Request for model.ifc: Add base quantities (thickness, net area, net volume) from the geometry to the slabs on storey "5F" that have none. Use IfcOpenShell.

First a look at what the model holds.

```python
import ifcopenshell
import ifcopenshell.util.element
import ifcopenshell.util.unit

model = ifcopenshell.open("model.ifc")
print(model.schema)
for unit_type in ("LENGTHUNIT", "AREAUNIT", "VOLUMEUNIT"):
    print(unit_type, ifcopenshell.util.unit.calculate_unit_scale(model, unit_type))
storey = next(s for s in model.by_type("IfcBuildingStorey") if s.Name == "5F")
slabs = [e for e in ifcopenshell.util.element.get_decomposition(storey) if e.is_a("IfcSlab")]
for e in sorted(slabs, key=lambda e: e.id()):
    print(e.id(), e.is_a(), e.Name, list(ifcopenshell.util.element.get_psets(e, qtos_only=True)), sep=" | ")
```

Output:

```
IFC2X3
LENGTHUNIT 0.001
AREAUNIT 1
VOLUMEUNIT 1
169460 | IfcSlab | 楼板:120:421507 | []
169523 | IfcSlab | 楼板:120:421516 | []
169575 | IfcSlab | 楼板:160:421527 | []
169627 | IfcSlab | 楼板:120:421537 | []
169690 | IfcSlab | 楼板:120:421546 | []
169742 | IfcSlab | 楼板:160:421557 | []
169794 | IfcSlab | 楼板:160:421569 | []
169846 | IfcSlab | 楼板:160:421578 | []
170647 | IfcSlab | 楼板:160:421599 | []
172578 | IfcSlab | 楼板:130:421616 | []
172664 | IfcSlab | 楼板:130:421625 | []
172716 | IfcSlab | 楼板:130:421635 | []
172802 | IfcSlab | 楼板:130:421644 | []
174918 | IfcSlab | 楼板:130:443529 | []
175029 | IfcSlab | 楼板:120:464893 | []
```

```python
import ifcopenshell
import ifcopenshell.api.pset
import ifcopenshell.geom
import ifcopenshell.util.element
import ifcopenshell.util.shape
import ifcopenshell.util.unit

model = ifcopenshell.open("model.ifc")
unit_scale = ifcopenshell.util.unit.calculate_unit_scale(model)
area_scale = ifcopenshell.util.unit.calculate_unit_scale(model, "AREAUNIT")
volume_scale = ifcopenshell.util.unit.calculate_unit_scale(model, "VOLUMEUNIT")
settings = ifcopenshell.geom.settings()

storey = next(s for s in model.by_type("IfcBuildingStorey") if s.Name == "5F")
slabs = [e for e in ifcopenshell.util.element.get_decomposition(storey) if e.is_a("IfcSlab")]

for e in sorted(slabs, key=lambda e: e.id()):
    if ifcopenshell.util.element.get_psets(e, qtos_only=True, should_inherit=False):
        continue
    # Geometry comes back in metres, in the element's own axes.
    shape = ifcopenshell.geom.create_shape(settings, e)
    values = {
        "Width": ifcopenshell.util.shape.get_z(shape.geometry) / unit_scale,
        "NetArea": ifcopenshell.util.shape.get_footprint_area(shape.geometry) / area_scale,
        "NetVolume": ifcopenshell.util.shape.get_volume(shape.geometry) / volume_scale,
    }
    qto = ifcopenshell.api.pset.add_qto(model, product=e, name="BaseQuantities")
    ifcopenshell.api.pset.edit_qto(model, qto=qto, properties=values)
    print(e.id(), {k: round(v, 3) for k, v in values.items()})

model.write("model-out.ifc")
```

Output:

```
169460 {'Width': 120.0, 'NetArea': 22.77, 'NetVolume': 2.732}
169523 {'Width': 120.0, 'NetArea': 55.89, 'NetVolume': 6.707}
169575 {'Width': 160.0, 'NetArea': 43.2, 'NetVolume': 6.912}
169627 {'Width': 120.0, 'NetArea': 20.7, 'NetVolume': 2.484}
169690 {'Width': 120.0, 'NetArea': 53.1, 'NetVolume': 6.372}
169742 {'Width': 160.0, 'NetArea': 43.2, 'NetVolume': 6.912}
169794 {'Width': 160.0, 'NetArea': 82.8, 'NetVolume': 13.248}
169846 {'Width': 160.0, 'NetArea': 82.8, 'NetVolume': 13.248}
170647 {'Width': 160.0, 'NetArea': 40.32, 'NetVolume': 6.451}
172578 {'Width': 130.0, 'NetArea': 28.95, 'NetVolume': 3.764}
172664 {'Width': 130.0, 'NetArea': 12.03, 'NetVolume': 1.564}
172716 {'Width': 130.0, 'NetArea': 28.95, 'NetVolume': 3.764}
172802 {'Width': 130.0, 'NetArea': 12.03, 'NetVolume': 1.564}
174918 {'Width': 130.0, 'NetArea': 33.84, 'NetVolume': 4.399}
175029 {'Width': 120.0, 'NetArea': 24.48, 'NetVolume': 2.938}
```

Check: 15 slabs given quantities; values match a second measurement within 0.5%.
